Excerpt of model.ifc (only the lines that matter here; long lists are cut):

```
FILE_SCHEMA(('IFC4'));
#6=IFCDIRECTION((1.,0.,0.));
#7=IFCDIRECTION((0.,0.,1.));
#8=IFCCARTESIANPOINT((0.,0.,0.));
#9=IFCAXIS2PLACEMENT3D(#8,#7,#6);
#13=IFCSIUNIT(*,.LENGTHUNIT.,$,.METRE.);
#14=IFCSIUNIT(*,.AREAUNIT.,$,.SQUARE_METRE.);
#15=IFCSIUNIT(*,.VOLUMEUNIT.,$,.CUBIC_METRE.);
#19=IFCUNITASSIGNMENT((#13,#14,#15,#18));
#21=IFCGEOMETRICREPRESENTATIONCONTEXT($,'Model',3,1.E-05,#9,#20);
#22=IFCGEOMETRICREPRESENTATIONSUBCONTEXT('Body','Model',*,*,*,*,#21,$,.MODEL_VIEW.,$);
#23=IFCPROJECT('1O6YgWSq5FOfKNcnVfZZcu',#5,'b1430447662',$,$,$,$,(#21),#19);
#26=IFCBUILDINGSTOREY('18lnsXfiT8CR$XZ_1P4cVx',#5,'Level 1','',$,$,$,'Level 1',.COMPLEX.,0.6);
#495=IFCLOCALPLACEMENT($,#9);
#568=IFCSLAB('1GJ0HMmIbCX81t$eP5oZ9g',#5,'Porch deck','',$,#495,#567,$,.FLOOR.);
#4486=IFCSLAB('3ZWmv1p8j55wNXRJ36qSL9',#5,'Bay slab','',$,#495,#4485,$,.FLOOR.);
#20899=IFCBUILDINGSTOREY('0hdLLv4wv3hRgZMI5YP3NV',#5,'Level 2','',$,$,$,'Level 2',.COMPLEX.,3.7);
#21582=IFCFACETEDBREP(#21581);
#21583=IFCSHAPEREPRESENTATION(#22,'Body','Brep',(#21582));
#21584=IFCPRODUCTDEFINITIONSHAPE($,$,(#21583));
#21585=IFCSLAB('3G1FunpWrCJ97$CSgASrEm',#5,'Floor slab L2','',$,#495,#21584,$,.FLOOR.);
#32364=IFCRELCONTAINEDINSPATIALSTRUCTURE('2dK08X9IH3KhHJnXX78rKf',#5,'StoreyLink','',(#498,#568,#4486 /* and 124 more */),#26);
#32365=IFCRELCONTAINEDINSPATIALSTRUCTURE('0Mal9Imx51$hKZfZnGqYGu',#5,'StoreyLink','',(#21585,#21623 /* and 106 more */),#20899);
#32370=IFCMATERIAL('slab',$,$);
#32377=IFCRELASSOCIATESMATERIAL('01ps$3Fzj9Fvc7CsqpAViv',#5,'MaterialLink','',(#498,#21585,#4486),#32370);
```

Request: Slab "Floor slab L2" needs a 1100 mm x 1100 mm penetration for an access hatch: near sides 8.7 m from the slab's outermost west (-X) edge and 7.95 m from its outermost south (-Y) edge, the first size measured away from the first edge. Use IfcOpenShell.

```python
import numpy as np
import ifcopenshell
import ifcopenshell.api.feature
import ifcopenshell.api.geometry
import ifcopenshell.api.root
import ifcopenshell.geom
import ifcopenshell.util.placement
import ifcopenshell.util.representation
import ifcopenshell.util.shape
import ifcopenshell.util.unit

model = ifcopenshell.open("model.ifc")
unit_scale = ifcopenshell.util.unit.calculate_unit_scale(model)
settings = ifcopenshell.geom.settings()


def volume(element):
    """Net volume in cubic metres, openings subtracted."""
    shape = ifcopenshell.geom.create_shape(settings, element)
    return ifcopenshell.util.shape.get_volume(shape.geometry)


slab = model.by_guid("3G1FunpWrCJ97$CSgASrEm")
before = volume(slab)

# Extent in the slab's own axes, in metres. The edges named are its -X and -Y sides.
slab_shape = ifcopenshell.geom.create_shape(settings, slab)
vertices = ifcopenshell.util.shape.get_vertices(slab_shape.geometry)
x_min, y_min, bottom = vertices.min(axis=0)
top = vertices[:, 2].max()

opening = ifcopenshell.api.root.create_entity(model, ifc_class="IfcOpeningElement", name="Access hatch opening", predefined_type="OPENING")
context = ifcopenshell.util.representation.get_context(model, "Model", "Body", "MODEL_VIEW")
width, depth = 1.1, 1.1
outline = [(0.0, 0.0), (width, 0.0), (width, depth), (0.0, depth), (0.0, 0.0)]
# Overshoot both faces by 50 mm so the cut is clean.
shape = ifcopenshell.api.geometry.add_slab_representation(
    model, context=context, depth=top - bottom + 0.1, polyline=outline
)
ifcopenshell.api.geometry.assign_representation(model, product=opening, representation=shape)

matrix = ifcopenshell.util.placement.get_local_placement(slab.ObjectPlacement)
matrix[:, 3] = matrix @ np.append(np.array([x_min + 8.7, y_min + 7.95, bottom - 0.05]) / unit_scale, 1.0)
ifcopenshell.api.geometry.edit_object_placement(model, product=opening, matrix=matrix, is_si=False)
ifcopenshell.api.feature.add_feature(model, feature=opening, element=slab)

after = volume(slab)

print(f"slab volume {before:.3f} -> {after:.3f} m3")

model.write("model_rev.ifc")
```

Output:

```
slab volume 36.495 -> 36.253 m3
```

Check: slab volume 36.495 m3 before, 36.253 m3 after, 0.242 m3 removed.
